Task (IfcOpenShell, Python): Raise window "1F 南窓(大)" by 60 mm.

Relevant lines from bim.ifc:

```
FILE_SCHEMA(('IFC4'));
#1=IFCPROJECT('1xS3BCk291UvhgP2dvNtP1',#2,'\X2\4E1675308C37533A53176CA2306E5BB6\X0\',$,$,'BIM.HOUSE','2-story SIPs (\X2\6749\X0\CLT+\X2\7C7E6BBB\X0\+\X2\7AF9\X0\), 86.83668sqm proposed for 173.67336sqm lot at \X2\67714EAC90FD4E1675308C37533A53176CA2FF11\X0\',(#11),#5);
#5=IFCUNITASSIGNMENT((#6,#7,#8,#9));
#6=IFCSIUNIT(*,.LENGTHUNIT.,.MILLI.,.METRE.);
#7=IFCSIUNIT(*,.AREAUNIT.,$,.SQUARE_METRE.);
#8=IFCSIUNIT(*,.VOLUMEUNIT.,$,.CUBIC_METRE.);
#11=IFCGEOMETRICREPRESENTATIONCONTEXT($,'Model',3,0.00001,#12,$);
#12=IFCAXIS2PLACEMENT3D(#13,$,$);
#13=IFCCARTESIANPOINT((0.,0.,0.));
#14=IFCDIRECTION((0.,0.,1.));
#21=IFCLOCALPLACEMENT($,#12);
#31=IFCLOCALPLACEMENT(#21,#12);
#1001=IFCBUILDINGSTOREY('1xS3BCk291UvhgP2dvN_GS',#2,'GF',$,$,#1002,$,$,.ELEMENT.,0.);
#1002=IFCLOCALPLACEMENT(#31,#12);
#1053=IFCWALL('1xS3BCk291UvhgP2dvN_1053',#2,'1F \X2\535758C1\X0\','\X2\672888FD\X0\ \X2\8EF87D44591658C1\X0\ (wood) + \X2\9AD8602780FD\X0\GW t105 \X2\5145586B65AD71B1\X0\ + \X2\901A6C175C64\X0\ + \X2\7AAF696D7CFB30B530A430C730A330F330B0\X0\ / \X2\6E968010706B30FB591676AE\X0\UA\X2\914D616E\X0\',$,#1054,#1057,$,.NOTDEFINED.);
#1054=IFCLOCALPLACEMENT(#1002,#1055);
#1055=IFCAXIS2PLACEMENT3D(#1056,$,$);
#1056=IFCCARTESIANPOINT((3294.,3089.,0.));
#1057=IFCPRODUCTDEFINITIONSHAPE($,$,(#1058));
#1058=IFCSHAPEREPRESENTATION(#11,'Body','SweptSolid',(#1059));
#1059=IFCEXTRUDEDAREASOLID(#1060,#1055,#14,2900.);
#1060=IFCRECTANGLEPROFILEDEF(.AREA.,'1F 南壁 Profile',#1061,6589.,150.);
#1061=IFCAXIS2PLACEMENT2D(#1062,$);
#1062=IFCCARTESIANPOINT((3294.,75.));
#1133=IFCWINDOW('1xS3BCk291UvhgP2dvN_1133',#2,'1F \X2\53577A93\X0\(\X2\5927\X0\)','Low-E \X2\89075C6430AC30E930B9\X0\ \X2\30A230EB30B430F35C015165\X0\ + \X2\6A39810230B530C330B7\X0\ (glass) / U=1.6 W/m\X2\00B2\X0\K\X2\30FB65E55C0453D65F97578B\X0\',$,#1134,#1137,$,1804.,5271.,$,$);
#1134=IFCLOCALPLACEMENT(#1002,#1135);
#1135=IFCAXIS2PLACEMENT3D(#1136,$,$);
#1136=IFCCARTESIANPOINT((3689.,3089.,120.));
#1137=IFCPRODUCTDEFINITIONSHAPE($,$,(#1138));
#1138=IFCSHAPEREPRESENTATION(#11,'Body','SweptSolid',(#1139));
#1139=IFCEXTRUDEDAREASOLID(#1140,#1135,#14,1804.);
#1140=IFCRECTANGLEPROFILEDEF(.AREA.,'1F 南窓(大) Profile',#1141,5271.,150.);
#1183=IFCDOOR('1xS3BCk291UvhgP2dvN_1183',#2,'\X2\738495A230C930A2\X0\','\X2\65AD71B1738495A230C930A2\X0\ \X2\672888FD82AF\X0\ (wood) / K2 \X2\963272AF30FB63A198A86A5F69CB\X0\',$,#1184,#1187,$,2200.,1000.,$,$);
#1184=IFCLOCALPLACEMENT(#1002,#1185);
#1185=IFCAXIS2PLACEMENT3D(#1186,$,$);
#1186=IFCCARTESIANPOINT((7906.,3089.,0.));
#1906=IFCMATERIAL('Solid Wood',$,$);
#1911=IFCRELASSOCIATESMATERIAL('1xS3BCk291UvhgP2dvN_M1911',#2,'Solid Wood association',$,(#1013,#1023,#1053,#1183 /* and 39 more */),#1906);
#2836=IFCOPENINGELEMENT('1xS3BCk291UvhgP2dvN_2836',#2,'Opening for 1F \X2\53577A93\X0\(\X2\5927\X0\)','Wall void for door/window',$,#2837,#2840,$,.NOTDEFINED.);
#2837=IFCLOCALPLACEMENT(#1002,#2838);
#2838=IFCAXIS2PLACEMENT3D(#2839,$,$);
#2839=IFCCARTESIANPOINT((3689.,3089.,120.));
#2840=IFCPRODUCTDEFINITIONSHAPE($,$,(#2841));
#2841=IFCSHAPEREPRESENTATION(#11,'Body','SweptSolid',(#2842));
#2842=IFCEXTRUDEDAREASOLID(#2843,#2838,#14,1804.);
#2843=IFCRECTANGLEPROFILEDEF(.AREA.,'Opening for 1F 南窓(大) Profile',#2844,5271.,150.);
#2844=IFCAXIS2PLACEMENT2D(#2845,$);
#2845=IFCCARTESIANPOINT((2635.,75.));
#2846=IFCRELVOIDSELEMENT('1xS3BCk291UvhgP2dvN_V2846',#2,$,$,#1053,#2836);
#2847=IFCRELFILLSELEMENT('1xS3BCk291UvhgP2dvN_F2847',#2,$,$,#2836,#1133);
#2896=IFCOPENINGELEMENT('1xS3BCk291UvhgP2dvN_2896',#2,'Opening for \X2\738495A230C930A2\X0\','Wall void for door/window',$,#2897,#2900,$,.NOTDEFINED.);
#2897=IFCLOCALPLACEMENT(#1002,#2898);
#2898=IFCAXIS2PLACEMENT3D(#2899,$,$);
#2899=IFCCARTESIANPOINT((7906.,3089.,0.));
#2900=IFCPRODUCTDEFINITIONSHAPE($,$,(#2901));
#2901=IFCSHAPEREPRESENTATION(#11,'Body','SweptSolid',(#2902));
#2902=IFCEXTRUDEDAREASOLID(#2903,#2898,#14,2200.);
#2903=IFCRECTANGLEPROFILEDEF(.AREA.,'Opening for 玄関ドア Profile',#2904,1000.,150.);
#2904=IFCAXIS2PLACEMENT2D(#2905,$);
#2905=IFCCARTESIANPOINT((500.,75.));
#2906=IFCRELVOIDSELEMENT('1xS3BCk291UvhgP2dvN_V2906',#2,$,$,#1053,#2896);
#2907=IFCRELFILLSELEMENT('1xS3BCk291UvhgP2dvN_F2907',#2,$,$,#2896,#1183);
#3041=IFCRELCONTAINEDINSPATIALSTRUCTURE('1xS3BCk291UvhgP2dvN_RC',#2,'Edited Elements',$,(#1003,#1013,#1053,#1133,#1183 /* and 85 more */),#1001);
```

```python
import numpy as np
import ifcopenshell
import ifcopenshell.api.geometry
import ifcopenshell.util.placement
import ifcopenshell.util.unit

model = ifcopenshell.open("bim.ifc")
unit_scale = ifcopenshell.util.unit.calculate_unit_scale(model)

window = model.by_guid("1xS3BCk291UvhgP2dvN_1133")
opening = window.FillsVoids[0].RelatingOpeningElement
dz = 60.0

shift = np.array([0.0, 0.0, dz])
# The window is not placed relative to its opening, so move both.
for product in (opening, window):
    matrix = ifcopenshell.util.placement.get_local_placement(product.ObjectPlacement)
    matrix[:3, 3] += shift
    ifcopenshell.api.geometry.edit_object_placement(model, product=product, matrix=matrix, is_si=False)

print(f"moved by {dz * unit_scale:+.3f} m")

model.write("bim-out.ifc")
```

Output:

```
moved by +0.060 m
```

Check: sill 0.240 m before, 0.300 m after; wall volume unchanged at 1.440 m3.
